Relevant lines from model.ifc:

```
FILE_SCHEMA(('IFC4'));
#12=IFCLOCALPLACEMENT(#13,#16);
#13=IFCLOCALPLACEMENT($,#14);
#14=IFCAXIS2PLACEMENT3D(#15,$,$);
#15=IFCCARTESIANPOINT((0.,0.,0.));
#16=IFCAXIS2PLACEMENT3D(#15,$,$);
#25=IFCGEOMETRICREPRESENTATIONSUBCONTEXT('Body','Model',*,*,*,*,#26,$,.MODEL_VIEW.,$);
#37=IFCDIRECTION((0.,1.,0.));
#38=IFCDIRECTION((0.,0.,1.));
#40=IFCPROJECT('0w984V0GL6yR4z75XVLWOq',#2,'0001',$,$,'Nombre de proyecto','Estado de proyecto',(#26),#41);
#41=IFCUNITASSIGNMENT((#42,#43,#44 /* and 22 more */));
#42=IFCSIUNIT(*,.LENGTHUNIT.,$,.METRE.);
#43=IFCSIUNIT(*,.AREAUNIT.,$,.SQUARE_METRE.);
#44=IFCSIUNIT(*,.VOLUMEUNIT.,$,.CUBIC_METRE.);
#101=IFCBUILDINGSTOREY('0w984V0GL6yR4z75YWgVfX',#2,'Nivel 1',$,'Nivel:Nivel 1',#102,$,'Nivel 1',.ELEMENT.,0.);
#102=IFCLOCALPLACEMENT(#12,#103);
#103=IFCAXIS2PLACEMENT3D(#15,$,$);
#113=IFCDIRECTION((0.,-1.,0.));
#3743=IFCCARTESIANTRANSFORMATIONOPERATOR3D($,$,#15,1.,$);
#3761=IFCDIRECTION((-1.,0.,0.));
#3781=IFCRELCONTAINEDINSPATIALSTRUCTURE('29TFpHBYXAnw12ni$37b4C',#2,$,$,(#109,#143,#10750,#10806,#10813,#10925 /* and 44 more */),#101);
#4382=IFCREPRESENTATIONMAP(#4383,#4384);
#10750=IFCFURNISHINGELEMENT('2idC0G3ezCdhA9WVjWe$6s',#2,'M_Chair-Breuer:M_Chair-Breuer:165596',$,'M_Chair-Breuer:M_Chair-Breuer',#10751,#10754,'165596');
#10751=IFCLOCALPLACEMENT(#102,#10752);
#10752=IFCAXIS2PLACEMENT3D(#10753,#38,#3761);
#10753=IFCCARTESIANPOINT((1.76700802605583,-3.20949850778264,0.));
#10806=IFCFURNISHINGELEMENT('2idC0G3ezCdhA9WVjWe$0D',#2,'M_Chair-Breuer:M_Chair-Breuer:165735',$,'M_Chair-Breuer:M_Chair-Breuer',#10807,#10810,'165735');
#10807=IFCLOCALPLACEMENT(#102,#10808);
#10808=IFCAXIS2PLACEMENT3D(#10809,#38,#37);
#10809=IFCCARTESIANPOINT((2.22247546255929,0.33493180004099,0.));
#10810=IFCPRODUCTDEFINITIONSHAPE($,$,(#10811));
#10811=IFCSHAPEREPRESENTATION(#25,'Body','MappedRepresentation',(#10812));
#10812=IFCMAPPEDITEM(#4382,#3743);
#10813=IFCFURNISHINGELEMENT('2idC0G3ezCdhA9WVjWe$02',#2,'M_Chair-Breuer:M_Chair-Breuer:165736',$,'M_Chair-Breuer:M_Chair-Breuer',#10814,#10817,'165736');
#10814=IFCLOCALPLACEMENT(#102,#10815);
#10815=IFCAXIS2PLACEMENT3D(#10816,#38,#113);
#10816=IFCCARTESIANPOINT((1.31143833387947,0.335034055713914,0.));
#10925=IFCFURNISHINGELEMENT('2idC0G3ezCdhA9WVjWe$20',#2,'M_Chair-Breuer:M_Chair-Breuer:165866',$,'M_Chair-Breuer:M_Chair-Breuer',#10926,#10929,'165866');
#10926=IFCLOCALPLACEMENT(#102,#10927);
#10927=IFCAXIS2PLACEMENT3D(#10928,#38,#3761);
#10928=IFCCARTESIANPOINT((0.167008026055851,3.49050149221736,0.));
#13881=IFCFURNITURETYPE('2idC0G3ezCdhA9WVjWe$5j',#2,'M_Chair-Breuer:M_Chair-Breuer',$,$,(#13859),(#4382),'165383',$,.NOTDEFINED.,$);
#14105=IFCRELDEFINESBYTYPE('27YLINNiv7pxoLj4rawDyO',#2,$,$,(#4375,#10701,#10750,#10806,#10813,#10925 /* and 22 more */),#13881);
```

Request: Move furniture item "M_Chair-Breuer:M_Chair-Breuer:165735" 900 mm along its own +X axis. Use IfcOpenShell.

```python
import ifcopenshell
import ifcopenshell.api.geometry
import ifcopenshell.util.placement

model = ifcopenshell.open("model.ifc")

item = model.by_id(10806)
matrix = ifcopenshell.util.placement.get_local_placement(item.ObjectPlacement)
matrix[:3, 3] += matrix[:3, 0] * 0.9
ifcopenshell.api.geometry.edit_object_placement(model, product=item, matrix=matrix, is_si=False)

print(ifcopenshell.util.placement.get_local_placement(item.ObjectPlacement).round(3) + 0.0)

model.write("model_rev.ifc")
```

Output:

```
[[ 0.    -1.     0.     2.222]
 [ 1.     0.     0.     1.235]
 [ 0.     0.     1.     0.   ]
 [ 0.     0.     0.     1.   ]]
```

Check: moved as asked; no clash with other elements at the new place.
